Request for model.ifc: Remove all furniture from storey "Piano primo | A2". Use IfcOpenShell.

First a look at what the model holds.

```python
import ifcopenshell
import ifcopenshell.util.element

model = ifcopenshell.open("model.ifc")
print(model.schema)
storey = next(s for s in model.by_type("IfcBuildingStorey") if s.Name == "Piano primo | A2")
furniture = [e for e in ifcopenshell.util.element.get_decomposition(storey) if e.is_a("IfcFurnishingElement")]
seen = {}
for e in furniture:
    element_type = ifcopenshell.util.element.get_type(e)
    name = element_type.Name if element_type not in (None, e) else None
    seen[name] = seen.get(name, 0) + 1
for name, count in sorted(seen.items(), key=str):
    print(count, "x", name)
```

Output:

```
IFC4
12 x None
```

```python
import ifcopenshell
import ifcopenshell.api.root
import ifcopenshell.util.element

model = ifcopenshell.open("model.ifc")

storey = next(s for s in model.by_type("IfcBuildingStorey") if s.Name == "Piano primo | A2")
furniture = [e for e in ifcopenshell.util.element.get_decomposition(storey) if e.is_a("IfcFurnishingElement")]

for e in furniture:
    ifcopenshell.api.root.remove_product(model, product=e)
print(len(furniture), "removed")

model.write("model_edited.ifc")
```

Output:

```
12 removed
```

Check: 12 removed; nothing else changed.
